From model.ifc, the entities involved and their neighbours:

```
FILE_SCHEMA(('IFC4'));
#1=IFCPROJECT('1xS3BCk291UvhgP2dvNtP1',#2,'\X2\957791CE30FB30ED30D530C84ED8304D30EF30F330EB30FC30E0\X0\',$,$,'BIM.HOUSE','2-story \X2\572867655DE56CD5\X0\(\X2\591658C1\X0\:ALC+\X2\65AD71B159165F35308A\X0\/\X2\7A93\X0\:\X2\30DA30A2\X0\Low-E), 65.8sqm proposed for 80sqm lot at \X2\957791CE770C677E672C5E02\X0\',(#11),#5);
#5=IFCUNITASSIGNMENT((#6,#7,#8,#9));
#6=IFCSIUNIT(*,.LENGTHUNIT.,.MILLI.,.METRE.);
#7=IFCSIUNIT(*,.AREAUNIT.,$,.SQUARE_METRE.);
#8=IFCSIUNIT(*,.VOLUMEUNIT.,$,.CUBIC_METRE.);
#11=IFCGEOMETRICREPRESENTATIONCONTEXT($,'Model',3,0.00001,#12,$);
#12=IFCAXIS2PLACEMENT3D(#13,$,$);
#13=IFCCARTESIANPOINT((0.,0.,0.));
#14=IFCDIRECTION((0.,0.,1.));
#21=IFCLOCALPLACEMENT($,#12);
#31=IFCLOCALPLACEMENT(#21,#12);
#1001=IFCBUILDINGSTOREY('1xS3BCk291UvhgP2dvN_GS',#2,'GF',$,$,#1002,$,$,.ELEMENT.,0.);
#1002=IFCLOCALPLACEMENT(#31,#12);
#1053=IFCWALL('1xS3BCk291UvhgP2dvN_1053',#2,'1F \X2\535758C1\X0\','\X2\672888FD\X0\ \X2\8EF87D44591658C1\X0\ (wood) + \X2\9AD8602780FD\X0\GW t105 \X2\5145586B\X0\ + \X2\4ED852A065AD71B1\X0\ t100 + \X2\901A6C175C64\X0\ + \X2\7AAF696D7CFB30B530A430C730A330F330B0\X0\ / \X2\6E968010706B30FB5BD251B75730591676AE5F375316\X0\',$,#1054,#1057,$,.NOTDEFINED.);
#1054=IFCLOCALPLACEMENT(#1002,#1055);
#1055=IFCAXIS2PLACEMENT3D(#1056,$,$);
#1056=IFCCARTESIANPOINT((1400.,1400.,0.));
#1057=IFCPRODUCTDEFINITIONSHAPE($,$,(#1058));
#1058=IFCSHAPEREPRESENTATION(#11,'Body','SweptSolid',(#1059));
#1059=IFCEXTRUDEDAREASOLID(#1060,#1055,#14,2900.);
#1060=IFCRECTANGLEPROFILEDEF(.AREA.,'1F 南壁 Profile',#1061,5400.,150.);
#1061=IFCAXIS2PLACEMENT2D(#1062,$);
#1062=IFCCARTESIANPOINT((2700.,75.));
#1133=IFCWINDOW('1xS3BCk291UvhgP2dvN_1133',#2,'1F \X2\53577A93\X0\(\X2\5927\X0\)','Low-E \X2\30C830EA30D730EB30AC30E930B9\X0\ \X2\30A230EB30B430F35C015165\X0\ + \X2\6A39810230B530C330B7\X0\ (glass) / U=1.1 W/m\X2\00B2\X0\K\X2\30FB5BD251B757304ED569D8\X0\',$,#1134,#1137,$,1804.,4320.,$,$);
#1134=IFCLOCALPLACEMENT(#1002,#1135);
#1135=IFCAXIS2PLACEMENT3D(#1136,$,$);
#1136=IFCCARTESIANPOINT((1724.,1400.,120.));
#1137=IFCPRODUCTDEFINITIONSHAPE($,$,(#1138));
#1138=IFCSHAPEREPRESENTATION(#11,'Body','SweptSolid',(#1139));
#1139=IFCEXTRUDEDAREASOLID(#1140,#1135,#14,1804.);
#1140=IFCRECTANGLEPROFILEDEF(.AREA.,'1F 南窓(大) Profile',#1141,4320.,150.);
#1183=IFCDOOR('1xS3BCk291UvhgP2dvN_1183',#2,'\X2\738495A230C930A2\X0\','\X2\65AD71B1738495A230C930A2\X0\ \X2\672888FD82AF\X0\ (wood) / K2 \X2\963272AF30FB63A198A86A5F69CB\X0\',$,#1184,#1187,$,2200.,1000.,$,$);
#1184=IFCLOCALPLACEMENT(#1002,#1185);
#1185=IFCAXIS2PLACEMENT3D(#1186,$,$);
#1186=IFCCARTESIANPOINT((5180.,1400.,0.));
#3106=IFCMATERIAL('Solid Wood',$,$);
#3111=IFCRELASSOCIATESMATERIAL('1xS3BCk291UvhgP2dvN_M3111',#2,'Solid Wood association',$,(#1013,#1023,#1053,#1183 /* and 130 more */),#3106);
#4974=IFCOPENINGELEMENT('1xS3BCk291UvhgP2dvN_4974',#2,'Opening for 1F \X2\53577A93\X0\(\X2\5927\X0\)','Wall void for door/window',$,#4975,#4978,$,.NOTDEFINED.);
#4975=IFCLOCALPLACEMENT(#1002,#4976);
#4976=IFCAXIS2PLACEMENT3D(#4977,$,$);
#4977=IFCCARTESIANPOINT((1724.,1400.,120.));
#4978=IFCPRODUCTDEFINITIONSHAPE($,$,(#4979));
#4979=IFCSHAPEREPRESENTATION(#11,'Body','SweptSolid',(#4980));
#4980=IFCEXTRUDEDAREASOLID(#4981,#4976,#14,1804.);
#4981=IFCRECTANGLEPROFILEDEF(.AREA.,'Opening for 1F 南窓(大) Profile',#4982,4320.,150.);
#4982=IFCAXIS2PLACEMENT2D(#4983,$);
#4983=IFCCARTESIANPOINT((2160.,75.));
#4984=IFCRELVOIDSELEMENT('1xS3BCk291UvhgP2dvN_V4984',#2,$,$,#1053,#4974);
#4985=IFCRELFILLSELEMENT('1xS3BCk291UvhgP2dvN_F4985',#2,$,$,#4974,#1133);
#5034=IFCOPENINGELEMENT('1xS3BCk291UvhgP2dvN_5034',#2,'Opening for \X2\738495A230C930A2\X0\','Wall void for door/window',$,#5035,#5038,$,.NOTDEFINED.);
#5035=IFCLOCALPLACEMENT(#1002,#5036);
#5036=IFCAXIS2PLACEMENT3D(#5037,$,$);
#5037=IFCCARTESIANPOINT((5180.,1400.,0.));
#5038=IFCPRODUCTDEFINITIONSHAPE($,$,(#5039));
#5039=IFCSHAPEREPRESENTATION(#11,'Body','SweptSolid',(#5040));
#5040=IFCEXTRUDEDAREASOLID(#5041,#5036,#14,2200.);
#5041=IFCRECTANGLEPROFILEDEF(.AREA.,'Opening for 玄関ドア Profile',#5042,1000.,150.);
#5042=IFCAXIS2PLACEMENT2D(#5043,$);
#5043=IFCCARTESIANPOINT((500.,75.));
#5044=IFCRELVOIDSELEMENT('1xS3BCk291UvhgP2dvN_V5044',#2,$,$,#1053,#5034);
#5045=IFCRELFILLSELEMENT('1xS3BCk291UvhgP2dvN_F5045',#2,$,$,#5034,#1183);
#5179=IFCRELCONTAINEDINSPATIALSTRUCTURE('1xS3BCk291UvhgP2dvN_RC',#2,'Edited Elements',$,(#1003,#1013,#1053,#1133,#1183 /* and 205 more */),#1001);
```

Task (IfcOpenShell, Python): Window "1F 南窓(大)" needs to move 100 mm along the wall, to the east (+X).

```python
import ifcopenshell
import ifcopenshell.api.geometry
import ifcopenshell.util.placement
import ifcopenshell.util.unit

model = ifcopenshell.open("model.ifc")
unit_scale = ifcopenshell.util.unit.calculate_unit_scale(model)

window = model.by_guid("1xS3BCk291UvhgP2dvN_1133")
opening = window.FillsVoids[0].RelatingOpeningElement
wall = opening.VoidsElements[0].RelatingBuildingElement

wall_matrix = ifcopenshell.util.placement.get_local_placement(wall.ObjectPlacement)
shift = wall_matrix[:3, 0] * 0.1 / unit_scale
before = ifcopenshell.util.placement.get_local_placement(window.ObjectPlacement)[:3, 3].copy()

# The window is not placed relative to its opening, so move both.
for product in (opening, window):
    matrix = ifcopenshell.util.placement.get_local_placement(product.ObjectPlacement)
    matrix[:3, 3] += shift
    ifcopenshell.api.geometry.edit_object_placement(model, product=product, matrix=matrix, is_si=False)

after = ifcopenshell.util.placement.get_local_placement(window.ObjectPlacement)[:3, 3]
print("window moved by", (after - before).round(3) + 0.0)

model.write("model_v2.ifc")
```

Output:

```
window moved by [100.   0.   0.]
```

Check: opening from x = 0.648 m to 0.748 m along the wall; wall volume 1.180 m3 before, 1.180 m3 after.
